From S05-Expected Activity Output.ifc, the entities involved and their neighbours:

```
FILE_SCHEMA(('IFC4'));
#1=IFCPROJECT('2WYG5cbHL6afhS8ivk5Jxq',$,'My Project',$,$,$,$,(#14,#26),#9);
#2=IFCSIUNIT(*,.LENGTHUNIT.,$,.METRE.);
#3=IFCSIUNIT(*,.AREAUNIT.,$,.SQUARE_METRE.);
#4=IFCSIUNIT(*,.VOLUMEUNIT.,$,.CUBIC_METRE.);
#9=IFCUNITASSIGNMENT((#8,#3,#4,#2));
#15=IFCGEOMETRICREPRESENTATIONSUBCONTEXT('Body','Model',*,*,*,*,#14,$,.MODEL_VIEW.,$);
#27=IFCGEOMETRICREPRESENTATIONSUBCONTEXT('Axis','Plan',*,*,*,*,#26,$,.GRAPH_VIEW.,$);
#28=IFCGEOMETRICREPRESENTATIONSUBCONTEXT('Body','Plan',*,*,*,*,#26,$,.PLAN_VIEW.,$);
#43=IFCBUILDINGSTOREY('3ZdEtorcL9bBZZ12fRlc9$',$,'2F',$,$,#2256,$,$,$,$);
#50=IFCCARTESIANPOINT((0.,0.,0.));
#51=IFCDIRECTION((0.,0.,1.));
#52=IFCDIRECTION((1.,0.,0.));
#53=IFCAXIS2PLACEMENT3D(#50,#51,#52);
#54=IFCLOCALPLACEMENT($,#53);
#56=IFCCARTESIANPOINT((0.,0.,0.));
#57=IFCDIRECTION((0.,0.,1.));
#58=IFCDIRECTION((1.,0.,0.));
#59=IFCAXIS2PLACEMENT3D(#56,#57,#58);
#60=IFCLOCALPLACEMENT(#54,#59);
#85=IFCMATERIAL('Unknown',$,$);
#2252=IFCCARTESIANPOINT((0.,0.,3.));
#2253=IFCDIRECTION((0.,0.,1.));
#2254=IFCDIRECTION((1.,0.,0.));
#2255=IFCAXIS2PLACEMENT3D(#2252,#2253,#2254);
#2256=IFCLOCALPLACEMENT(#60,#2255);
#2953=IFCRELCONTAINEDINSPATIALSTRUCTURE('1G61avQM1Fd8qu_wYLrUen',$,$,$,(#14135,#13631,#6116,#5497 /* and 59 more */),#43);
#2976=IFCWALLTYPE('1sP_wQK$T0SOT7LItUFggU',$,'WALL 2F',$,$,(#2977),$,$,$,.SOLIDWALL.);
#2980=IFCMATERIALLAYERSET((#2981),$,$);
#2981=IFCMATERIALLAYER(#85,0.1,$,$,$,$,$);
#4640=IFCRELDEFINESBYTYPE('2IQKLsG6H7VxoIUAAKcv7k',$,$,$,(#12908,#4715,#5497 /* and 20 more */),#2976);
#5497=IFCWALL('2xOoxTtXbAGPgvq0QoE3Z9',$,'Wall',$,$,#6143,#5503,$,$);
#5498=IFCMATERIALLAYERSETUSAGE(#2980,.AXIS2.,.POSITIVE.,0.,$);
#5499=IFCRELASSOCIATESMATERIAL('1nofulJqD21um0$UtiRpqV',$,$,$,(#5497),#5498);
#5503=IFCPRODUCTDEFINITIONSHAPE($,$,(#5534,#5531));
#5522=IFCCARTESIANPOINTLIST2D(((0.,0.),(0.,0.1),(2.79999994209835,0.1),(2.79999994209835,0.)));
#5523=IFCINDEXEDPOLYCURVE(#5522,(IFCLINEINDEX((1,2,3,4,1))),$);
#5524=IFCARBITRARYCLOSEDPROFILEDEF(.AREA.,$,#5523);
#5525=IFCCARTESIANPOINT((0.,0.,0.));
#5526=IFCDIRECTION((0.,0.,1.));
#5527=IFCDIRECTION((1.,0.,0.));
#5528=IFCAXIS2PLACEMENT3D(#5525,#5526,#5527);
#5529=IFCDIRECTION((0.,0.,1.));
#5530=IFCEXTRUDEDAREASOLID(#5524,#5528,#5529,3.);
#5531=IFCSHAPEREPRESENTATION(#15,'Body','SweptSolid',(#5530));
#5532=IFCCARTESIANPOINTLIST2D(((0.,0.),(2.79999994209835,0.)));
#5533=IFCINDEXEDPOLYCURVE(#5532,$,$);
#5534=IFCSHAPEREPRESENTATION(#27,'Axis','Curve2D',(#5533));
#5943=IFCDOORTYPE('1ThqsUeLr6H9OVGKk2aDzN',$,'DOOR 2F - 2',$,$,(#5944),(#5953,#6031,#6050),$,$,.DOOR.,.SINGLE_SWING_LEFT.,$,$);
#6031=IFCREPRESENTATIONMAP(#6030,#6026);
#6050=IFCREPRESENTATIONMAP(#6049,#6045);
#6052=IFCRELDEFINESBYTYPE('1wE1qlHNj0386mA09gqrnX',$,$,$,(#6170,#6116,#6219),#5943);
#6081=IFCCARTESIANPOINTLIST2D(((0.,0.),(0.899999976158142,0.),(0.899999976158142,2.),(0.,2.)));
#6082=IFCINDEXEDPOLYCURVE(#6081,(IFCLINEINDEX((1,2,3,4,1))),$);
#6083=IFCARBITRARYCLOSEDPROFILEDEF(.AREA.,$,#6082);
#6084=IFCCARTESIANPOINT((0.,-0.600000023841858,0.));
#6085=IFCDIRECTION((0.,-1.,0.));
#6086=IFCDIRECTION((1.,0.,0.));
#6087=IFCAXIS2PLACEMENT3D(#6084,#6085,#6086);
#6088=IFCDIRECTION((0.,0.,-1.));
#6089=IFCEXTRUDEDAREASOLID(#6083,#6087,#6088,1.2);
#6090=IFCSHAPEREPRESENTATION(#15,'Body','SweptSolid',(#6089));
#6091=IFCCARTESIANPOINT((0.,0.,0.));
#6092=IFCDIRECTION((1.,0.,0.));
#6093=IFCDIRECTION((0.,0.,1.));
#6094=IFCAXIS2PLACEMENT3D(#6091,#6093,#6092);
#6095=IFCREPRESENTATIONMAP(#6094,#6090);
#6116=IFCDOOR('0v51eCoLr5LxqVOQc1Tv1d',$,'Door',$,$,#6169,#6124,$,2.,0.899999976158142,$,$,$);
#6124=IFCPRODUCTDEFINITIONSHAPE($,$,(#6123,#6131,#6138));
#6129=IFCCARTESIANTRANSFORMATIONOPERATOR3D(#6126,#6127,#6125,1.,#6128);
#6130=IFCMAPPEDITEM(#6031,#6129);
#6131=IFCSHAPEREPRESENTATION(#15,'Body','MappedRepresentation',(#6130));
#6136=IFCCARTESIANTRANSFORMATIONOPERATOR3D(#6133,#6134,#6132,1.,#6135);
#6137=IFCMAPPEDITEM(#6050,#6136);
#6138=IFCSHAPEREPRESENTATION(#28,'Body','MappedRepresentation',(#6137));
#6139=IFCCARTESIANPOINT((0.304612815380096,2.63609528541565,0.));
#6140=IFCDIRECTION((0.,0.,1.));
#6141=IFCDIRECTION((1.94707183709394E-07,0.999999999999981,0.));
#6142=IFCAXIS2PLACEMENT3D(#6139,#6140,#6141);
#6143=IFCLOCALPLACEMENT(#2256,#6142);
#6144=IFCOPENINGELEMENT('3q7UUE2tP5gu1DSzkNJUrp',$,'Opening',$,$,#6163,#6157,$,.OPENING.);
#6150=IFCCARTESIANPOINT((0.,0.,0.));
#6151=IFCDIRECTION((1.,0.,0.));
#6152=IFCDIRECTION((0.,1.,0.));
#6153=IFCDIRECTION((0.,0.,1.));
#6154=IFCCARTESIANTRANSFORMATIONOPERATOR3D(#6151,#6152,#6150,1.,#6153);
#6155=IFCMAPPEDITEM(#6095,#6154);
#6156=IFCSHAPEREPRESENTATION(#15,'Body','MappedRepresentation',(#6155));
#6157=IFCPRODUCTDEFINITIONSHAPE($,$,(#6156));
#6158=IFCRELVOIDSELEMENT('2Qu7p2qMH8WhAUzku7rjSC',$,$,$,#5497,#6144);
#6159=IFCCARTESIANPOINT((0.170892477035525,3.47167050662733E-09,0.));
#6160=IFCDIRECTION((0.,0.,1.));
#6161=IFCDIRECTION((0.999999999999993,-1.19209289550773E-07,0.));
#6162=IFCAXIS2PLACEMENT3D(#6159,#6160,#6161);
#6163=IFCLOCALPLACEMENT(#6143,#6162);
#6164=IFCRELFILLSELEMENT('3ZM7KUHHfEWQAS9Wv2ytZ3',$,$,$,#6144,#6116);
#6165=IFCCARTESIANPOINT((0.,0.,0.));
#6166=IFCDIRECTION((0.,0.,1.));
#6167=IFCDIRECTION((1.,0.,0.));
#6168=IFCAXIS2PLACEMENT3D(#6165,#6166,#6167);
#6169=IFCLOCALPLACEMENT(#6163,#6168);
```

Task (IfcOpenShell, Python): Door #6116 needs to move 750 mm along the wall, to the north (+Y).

```python
import ifcopenshell
import ifcopenshell.api.geometry
import ifcopenshell.util.placement

model = ifcopenshell.open("S05-Expected Activity Output.ifc")

door = model.by_id(6116)
opening = door.FillsVoids[0].RelatingOpeningElement
wall = opening.VoidsElements[0].RelatingBuildingElement

wall_matrix = ifcopenshell.util.placement.get_local_placement(wall.ObjectPlacement)
shift = wall_matrix[:3, 0] * 0.75
before = ifcopenshell.util.placement.get_local_placement(door.ObjectPlacement)[:3, 3].copy()

# The door is placed relative to its opening, so it follows when the opening moves.
matrix = ifcopenshell.util.placement.get_local_placement(opening.ObjectPlacement)
matrix[:3, 3] += shift
ifcopenshell.api.geometry.edit_object_placement(
    model, product=opening, matrix=matrix, is_si=False, should_transform_children=True
)

after = ifcopenshell.util.placement.get_local_placement(door.ObjectPlacement)[:3, 3]
print("door moved by", (after - before).round(3) + 0.0)

model.write("S05-Expected Activity Output_updated.ifc")
```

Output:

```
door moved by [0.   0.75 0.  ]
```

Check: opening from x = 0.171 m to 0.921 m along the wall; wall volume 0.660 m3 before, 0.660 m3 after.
